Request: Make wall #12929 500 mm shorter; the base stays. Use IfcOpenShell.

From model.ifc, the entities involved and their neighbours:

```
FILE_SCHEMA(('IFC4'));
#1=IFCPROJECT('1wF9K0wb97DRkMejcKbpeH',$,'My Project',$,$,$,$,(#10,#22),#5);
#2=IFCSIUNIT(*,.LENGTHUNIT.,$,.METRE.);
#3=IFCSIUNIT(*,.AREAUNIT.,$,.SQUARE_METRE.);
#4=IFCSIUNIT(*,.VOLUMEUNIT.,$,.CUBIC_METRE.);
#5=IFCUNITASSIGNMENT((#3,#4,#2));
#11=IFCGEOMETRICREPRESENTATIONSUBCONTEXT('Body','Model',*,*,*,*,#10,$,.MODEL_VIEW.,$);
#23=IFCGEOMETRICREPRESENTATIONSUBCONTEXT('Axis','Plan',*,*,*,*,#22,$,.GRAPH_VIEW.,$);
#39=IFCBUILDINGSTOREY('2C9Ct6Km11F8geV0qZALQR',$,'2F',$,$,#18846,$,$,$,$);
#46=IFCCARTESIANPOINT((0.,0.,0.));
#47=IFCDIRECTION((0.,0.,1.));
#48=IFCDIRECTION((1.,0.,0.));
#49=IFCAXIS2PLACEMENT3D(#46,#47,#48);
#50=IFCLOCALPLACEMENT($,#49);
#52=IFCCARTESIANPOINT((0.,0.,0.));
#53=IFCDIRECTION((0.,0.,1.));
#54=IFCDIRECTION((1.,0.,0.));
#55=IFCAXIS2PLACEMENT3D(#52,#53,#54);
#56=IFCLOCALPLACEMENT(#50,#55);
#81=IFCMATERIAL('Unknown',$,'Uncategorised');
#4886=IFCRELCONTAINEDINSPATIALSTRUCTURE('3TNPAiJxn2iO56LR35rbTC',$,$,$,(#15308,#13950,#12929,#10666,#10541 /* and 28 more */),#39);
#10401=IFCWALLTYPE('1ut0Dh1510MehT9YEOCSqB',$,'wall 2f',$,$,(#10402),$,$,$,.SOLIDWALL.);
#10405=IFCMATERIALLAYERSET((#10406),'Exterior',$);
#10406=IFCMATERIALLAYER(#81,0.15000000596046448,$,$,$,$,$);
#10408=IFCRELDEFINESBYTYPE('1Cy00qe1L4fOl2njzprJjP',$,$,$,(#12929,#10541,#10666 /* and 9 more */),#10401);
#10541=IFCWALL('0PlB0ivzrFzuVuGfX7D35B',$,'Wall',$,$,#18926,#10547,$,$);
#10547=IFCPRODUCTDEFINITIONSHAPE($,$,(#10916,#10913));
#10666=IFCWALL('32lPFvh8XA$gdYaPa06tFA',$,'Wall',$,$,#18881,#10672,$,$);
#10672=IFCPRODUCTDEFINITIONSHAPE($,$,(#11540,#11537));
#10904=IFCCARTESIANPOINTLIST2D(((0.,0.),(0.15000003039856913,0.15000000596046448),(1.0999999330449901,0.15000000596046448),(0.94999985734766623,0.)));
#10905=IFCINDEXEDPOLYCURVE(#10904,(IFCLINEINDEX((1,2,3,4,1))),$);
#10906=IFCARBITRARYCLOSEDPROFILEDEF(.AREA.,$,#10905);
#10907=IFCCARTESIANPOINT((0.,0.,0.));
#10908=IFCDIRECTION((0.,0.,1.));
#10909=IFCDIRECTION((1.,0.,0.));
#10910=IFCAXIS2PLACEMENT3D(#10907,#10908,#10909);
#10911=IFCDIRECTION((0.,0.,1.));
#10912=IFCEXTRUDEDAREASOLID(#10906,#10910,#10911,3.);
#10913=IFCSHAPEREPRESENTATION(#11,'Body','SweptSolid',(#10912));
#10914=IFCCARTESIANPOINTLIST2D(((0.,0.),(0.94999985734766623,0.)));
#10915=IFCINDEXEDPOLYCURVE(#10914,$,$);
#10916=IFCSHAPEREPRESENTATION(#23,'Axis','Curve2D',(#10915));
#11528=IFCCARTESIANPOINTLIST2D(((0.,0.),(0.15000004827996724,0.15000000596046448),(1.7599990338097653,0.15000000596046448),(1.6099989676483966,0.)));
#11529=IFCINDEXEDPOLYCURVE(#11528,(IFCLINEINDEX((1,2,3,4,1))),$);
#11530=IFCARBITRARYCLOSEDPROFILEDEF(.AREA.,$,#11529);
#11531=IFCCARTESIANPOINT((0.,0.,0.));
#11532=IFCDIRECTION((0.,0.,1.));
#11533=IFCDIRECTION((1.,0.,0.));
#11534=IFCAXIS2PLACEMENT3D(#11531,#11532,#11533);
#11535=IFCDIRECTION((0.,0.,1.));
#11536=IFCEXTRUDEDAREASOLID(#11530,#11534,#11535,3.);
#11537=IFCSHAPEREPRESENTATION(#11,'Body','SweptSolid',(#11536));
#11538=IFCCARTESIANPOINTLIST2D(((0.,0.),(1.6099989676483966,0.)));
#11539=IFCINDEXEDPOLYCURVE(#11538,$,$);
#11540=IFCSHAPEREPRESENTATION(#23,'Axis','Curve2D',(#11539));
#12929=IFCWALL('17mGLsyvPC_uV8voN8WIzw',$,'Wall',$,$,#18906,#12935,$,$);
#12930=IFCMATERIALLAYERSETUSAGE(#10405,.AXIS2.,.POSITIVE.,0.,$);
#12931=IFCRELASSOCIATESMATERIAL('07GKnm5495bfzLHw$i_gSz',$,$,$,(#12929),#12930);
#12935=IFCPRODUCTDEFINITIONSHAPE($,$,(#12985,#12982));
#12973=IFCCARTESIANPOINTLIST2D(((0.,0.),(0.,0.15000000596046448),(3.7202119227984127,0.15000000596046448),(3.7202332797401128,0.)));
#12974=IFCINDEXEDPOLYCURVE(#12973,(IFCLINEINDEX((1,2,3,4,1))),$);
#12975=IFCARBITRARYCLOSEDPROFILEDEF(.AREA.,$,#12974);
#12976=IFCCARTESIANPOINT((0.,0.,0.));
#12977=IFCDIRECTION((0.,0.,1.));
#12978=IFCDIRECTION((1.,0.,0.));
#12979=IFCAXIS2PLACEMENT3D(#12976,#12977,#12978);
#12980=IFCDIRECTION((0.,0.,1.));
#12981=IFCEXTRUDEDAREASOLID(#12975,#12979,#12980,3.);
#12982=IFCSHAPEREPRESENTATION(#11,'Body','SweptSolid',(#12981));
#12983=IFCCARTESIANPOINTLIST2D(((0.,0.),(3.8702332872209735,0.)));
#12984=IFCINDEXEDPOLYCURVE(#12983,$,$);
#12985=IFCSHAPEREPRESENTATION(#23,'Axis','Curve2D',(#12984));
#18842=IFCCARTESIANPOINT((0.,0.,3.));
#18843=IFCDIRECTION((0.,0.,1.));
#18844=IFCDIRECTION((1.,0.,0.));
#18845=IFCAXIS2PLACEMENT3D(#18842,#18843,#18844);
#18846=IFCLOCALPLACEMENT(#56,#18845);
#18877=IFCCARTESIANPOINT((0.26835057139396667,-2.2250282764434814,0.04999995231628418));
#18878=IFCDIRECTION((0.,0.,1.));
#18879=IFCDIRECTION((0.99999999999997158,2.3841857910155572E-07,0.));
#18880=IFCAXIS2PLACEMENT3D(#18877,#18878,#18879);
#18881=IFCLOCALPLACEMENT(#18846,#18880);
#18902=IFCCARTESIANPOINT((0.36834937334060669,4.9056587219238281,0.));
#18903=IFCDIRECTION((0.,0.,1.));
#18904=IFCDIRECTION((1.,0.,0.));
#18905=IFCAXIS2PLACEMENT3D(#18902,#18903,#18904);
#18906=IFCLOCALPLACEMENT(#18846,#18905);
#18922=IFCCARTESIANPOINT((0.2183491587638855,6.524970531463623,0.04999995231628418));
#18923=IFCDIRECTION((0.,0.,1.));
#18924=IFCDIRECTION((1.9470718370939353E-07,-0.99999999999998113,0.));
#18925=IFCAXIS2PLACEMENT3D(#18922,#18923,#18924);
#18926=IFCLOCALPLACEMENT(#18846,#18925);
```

```python
import ifcopenshell
import ifcopenshell.geom
import ifcopenshell.util.representation
import ifcopenshell.util.shape

model = ifcopenshell.open("model.ifc")
settings = ifcopenshell.geom.settings()


def volume(element):
    """Net volume in cubic metres, openings subtracted."""
    shape = ifcopenshell.geom.create_shape(settings, element)
    return ifcopenshell.util.shape.get_volume(shape.geometry)


wall = model.by_id(12929)
before = volume(wall)

body = ifcopenshell.util.representation.get_representation(wall, "Model", "Body")
solid = body.Items[0]
old_height = solid.Depth
solid.Depth -= 0.5
after = volume(wall)

print(f"height {old_height:g} -> {solid.Depth:g}, volume {before:.3f} -> {after:.3f} m3")

model.write("model_edited.ifc")
```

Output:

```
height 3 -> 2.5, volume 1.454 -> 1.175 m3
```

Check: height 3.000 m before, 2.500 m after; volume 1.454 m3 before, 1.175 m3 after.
